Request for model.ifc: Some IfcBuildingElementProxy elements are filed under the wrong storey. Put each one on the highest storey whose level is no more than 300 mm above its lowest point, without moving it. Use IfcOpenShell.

First a look at what the model holds.

```python
import ifcopenshell
import ifcopenshell.util.element
import ifcopenshell.util.placement

model = ifcopenshell.open("model.ifc")
print(model.schema)
for storey in model.by_type("IfcBuildingStorey"):
    level = ifcopenshell.util.placement.get_storey_elevation(storey)
    count = sum(e.is_a("IfcBuildingElementProxy") for e in ifcopenshell.util.element.get_contained(storey))
    print(storey.id(), storey.Name, round(level, 3), count, sep=" | ")
```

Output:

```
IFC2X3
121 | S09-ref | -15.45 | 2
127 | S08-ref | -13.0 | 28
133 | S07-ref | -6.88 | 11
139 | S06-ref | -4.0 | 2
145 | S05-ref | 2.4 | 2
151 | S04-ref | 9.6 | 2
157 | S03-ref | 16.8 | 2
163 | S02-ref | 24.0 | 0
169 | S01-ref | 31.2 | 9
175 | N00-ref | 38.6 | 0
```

```python
import ifcopenshell
import ifcopenshell.api.spatial
import ifcopenshell.geom
import ifcopenshell.util.element
import ifcopenshell.util.placement
import ifcopenshell.util.shape
import ifcopenshell.util.unit

model = ifcopenshell.open("model.ifc")
unit_scale = ifcopenshell.util.unit.calculate_unit_scale(model)
settings = ifcopenshell.geom.settings()

levels = sorted(
    ((ifcopenshell.util.placement.get_storey_elevation(s) * unit_scale, s) for s in model.by_type("IfcBuildingStorey")),
    key=lambda pair: pair[0],
)

for e in model.by_type("IfcBuildingElementProxy"):
    current = e.ContainedInStructure[0].RelatingStructure if e.ContainedInStructure else None
    if current is None or not current.is_a("IfcBuildingStorey"):
        continue
    shape = ifcopenshell.geom.create_shape(settings, e)
    bottom = ifcopenshell.util.shape.get_shape_bottom_elevation(shape, shape.geometry)
    below = [s for level, s in levels if level <= bottom + 0.3]
    storey = below[-1] if below else levels[0][1]
    if storey != current:
        # assign_container keeps the world position.
        ifcopenshell.api.spatial.assign_container(model, products=[e], relating_structure=storey)
        print(e.id(), current.Name, "->", storey.Name)

model.write("model_v2.ifc")
```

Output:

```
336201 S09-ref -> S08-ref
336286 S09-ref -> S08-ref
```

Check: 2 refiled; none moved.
